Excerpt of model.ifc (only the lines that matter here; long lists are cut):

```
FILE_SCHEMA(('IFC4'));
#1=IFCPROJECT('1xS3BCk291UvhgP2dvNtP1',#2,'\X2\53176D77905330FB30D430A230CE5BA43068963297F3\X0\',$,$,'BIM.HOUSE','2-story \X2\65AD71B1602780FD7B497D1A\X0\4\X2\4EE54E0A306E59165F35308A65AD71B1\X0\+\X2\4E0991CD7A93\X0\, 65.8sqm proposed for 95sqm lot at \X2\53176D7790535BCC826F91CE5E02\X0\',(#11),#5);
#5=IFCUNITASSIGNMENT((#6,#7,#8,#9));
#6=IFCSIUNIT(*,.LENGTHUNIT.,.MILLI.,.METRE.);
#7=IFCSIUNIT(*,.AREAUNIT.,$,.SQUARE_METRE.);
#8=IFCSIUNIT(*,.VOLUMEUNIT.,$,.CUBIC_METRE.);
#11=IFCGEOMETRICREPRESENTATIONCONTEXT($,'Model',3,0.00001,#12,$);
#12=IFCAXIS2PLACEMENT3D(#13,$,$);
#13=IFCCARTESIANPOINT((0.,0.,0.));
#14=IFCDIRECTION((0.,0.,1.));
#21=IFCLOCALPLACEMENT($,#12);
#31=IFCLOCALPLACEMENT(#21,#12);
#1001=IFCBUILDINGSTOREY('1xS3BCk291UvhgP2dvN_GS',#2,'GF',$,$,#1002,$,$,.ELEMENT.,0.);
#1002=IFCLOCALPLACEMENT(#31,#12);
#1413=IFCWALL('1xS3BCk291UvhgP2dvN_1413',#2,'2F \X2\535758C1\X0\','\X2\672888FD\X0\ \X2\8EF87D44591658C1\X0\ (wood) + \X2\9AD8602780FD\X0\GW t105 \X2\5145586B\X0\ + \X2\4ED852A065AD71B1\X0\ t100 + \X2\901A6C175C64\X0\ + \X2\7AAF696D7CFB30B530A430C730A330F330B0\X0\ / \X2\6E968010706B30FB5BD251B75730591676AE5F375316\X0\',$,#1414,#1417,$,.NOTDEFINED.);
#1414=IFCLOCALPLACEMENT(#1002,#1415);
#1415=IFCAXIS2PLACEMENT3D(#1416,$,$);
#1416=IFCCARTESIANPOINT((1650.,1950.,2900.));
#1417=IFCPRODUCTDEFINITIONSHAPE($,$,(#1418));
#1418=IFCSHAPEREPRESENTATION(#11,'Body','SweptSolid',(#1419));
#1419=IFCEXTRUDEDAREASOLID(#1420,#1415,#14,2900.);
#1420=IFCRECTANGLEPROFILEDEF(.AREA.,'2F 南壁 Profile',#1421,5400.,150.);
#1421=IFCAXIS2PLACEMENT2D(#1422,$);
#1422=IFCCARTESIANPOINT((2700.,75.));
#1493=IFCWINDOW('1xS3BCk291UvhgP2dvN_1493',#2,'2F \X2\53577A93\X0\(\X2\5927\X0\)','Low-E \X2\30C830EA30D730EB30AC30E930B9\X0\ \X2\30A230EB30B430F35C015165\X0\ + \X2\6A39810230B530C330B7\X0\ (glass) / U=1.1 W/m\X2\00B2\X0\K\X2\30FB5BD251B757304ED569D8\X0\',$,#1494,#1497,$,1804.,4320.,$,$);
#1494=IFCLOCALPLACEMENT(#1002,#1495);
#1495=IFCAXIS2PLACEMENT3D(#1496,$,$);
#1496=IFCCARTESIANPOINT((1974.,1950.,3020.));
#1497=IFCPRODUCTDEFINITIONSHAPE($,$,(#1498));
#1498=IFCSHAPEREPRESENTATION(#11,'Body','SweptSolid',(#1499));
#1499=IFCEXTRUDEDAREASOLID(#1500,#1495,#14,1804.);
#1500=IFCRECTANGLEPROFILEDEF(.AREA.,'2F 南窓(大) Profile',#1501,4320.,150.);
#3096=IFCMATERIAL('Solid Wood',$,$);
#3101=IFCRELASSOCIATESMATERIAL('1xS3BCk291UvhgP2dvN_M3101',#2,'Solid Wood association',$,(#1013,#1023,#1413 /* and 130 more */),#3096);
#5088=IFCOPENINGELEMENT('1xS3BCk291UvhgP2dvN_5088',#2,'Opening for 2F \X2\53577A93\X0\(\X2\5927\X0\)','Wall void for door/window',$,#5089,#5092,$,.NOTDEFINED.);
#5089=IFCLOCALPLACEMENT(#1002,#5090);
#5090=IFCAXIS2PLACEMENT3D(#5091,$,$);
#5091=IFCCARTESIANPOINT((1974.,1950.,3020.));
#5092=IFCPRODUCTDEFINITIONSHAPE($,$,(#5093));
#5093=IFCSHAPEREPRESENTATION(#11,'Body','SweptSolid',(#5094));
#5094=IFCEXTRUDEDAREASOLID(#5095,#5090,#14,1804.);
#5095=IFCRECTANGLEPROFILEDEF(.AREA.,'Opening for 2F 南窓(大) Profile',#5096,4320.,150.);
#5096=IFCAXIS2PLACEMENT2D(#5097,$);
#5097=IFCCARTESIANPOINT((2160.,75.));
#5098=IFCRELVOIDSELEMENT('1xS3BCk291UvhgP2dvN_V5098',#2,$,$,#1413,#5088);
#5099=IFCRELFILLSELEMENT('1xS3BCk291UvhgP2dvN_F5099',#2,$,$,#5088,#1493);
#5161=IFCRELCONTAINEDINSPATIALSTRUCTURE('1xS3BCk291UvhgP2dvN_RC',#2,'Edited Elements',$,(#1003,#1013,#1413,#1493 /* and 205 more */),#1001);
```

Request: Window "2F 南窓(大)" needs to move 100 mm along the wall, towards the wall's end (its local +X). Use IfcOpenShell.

```python
import ifcopenshell
import ifcopenshell.api.geometry
import ifcopenshell.util.placement

model = ifcopenshell.open("model.ifc")

window = model.by_id(1493)
opening = window.FillsVoids[0].RelatingOpeningElement
wall = opening.VoidsElements[0].RelatingBuildingElement

wall_matrix = ifcopenshell.util.placement.get_local_placement(wall.ObjectPlacement)
shift = wall_matrix[:3, 0] * 100.0
before = ifcopenshell.util.placement.get_local_placement(window.ObjectPlacement)[:3, 3].copy()

# The window is not placed relative to its opening, so move both.
for product in (opening, window):
    matrix = ifcopenshell.util.placement.get_local_placement(product.ObjectPlacement)
    matrix[:3, 3] += shift
    ifcopenshell.api.geometry.edit_object_placement(model, product=product, matrix=matrix, is_si=False)

after = ifcopenshell.util.placement.get_local_placement(window.ObjectPlacement)[:3, 3]
print("window moved by", (after - before).round(3) + 0.0)

model.write("model_updated.ifc")
```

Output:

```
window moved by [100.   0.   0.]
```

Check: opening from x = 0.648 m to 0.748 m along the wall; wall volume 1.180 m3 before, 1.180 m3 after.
